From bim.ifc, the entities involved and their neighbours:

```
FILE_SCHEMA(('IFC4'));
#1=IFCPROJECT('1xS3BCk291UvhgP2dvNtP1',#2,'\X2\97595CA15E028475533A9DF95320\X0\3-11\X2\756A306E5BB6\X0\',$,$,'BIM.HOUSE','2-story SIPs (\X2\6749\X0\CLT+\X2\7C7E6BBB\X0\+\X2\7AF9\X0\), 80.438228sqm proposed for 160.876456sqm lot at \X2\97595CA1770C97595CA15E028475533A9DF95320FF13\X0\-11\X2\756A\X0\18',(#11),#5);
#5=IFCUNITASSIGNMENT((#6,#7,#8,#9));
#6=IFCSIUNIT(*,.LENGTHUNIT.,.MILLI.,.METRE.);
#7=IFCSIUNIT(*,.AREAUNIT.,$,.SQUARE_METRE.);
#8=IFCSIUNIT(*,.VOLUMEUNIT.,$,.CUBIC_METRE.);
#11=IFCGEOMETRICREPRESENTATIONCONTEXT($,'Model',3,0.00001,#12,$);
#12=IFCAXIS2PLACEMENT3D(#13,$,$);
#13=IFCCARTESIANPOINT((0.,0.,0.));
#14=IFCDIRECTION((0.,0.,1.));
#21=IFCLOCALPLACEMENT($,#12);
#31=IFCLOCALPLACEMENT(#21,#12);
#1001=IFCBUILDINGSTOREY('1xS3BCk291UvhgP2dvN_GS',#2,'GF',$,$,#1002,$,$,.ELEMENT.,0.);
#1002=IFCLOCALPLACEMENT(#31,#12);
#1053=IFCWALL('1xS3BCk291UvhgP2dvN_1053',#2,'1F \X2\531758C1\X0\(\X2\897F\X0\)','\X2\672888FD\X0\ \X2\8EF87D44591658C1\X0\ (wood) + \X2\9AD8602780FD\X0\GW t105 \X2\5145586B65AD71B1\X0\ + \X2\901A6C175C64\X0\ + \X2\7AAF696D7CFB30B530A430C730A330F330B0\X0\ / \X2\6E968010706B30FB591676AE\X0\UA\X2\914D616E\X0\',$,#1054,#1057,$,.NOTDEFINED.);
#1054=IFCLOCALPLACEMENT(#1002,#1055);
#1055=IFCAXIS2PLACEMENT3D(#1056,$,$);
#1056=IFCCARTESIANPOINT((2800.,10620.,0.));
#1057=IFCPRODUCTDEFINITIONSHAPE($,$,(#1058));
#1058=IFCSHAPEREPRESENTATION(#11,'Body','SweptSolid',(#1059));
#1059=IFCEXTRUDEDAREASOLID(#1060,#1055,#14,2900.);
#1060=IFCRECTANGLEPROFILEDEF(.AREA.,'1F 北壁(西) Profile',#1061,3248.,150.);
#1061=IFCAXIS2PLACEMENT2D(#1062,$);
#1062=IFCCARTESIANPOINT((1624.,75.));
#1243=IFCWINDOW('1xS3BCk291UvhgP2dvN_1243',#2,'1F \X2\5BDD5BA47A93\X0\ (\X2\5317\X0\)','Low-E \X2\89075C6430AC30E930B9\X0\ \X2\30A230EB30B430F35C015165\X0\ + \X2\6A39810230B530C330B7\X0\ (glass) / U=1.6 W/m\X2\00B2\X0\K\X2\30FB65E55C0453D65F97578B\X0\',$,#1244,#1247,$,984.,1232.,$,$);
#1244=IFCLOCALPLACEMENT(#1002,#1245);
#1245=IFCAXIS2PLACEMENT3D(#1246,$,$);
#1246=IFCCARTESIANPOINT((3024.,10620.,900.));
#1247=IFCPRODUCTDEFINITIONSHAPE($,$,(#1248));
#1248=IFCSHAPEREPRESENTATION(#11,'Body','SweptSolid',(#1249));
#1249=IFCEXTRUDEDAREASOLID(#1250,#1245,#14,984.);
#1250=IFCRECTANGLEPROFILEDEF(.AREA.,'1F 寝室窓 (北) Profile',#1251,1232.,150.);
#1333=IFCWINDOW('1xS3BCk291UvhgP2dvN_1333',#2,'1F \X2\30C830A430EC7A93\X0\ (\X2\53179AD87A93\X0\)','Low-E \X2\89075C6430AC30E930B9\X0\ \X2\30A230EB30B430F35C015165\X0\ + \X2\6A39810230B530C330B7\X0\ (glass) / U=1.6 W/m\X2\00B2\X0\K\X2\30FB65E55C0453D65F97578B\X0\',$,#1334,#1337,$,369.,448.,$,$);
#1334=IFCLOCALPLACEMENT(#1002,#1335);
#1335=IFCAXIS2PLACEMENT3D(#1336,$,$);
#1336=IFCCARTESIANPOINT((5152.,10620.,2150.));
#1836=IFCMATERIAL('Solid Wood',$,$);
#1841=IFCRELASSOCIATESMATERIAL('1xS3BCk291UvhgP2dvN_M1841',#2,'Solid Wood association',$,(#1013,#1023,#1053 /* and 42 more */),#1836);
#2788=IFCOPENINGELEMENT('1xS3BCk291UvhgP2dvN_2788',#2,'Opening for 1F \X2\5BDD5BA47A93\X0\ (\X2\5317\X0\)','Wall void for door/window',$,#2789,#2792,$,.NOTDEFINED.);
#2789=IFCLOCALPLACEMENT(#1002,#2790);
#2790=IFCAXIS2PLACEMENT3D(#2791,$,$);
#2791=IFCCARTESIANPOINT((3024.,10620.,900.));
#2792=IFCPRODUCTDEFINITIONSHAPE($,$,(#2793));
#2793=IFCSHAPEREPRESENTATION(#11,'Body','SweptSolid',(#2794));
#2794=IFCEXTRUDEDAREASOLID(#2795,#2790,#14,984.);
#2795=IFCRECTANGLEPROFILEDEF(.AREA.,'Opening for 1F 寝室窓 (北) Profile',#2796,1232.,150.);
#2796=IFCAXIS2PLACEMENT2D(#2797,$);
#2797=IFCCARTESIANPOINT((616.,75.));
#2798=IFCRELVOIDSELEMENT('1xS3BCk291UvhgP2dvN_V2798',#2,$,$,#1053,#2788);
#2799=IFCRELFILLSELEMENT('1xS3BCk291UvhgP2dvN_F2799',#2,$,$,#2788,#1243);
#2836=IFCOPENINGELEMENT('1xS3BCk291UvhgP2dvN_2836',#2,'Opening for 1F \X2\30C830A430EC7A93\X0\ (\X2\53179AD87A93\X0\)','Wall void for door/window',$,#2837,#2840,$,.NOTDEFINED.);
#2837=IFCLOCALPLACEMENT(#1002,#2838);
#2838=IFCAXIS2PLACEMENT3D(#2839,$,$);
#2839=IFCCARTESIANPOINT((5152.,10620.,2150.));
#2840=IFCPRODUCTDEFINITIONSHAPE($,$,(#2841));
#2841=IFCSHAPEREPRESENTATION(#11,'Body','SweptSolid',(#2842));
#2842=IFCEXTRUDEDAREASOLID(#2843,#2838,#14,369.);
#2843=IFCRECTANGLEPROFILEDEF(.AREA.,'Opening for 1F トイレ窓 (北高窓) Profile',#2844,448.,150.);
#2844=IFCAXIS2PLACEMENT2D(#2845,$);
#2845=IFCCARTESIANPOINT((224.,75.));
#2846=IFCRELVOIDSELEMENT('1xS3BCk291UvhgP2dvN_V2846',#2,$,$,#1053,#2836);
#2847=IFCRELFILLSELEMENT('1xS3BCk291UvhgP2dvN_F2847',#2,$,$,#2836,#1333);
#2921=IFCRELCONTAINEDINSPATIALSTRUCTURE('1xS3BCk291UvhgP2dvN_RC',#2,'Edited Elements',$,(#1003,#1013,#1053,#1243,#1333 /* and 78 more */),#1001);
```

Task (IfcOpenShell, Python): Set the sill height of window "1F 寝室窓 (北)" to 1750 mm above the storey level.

```python
import numpy as np
import ifcopenshell
import ifcopenshell.api.geometry
import ifcopenshell.geom
import ifcopenshell.util.element
import ifcopenshell.util.placement
import ifcopenshell.util.shape
import ifcopenshell.util.unit

model = ifcopenshell.open("bim.ifc")
unit_scale = ifcopenshell.util.unit.calculate_unit_scale(model)

window = model.by_guid("1xS3BCk291UvhgP2dvN_1243")
opening = window.FillsVoids[0].RelatingOpeningElement
storey = ifcopenshell.util.element.get_container(window, ifc_class="IfcBuildingStorey")
level = ifcopenshell.util.placement.get_local_placement(storey.ObjectPlacement)[2, 3]

# The opening's origin need not be at the sill, so measure its lowest point.
shape = ifcopenshell.geom.create_shape(ifcopenshell.geom.settings(), opening)
bottom = ifcopenshell.util.shape.get_shape_bottom_elevation(shape, shape.geometry) / unit_scale
dz = level + 1.75 / unit_scale - bottom

shift = np.array([0.0, 0.0, dz])
# The window is not placed relative to its opening, so move both.
for product in (opening, window):
    matrix = ifcopenshell.util.placement.get_local_placement(product.ObjectPlacement)
    matrix[:3, 3] += shift
    ifcopenshell.api.geometry.edit_object_placement(model, product=product, matrix=matrix, is_si=False)

print(f"moved by {dz * unit_scale:+.3f} m")

model.write("bim-out.ifc")
```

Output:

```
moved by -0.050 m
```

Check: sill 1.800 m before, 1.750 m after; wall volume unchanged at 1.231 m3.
